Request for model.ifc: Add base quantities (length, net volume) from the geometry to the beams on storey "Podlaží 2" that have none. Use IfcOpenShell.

First a look at what the model holds.

```python
import ifcopenshell
import ifcopenshell.util.element
import ifcopenshell.util.unit

model = ifcopenshell.open("model.ifc")
print(model.schema)
for unit_type in ("LENGTHUNIT", "AREAUNIT", "VOLUMEUNIT"):
    print(unit_type, ifcopenshell.util.unit.calculate_unit_scale(model, unit_type))
storey = next(s for s in model.by_type("IfcBuildingStorey") if s.Name == "Podlaží 2")
beams = [e for e in ifcopenshell.util.element.get_decomposition(storey) if e.is_a("IfcBeam")]
for e in sorted(beams, key=lambda e: e.id()):
    print(e.id(), e.is_a(), e.Name, list(ifcopenshell.util.element.get_psets(e, qtos_only=True)), sep=" | ")
```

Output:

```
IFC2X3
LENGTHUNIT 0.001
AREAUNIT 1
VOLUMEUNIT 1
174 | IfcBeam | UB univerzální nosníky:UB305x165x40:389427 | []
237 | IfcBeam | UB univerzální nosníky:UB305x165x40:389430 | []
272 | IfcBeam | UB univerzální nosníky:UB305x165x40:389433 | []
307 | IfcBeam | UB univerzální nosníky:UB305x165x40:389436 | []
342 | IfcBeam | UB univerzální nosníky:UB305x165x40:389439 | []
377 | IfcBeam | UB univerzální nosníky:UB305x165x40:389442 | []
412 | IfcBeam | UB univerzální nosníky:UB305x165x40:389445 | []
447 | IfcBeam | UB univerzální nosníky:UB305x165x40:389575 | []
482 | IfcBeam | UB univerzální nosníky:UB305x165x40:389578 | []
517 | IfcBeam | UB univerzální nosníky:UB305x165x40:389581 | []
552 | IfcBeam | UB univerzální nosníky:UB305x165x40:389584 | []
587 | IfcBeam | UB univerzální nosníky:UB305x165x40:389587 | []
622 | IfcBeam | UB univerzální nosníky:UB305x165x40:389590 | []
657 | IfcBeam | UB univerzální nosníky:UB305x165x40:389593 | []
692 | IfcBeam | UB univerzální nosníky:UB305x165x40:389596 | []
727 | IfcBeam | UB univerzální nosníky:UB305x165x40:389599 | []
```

```python
import ifcopenshell
import ifcopenshell.api.pset
import ifcopenshell.geom
import ifcopenshell.util.element
import ifcopenshell.util.shape
import ifcopenshell.util.unit

model = ifcopenshell.open("model.ifc")
unit_scale = ifcopenshell.util.unit.calculate_unit_scale(model)
volume_scale = ifcopenshell.util.unit.calculate_unit_scale(model, "VOLUMEUNIT")
settings = ifcopenshell.geom.settings()

storey = next(s for s in model.by_type("IfcBuildingStorey") if s.Name == "Podlaží 2")
beams = [e for e in ifcopenshell.util.element.get_decomposition(storey) if e.is_a("IfcBeam")]

for e in sorted(beams, key=lambda e: e.id()):
    if ifcopenshell.util.element.get_psets(e, qtos_only=True, should_inherit=False):
        continue
    # Geometry comes back in metres, in the element's own axes.
    shape = ifcopenshell.geom.create_shape(settings, e)
    values = {
        "Length": ifcopenshell.util.shape.get_max_xyz(shape.geometry) / unit_scale,
        "NetVolume": ifcopenshell.util.shape.get_volume(shape.geometry) / volume_scale,
    }
    qto = ifcopenshell.api.pset.add_qto(model, product=e, name="BaseQuantities")
    ifcopenshell.api.pset.edit_qto(model, qto=qto, properties=values)
    print(e.id(), {k: round(v, 3) for k, v in values.items()})

model.write("model_v2.ifc")
```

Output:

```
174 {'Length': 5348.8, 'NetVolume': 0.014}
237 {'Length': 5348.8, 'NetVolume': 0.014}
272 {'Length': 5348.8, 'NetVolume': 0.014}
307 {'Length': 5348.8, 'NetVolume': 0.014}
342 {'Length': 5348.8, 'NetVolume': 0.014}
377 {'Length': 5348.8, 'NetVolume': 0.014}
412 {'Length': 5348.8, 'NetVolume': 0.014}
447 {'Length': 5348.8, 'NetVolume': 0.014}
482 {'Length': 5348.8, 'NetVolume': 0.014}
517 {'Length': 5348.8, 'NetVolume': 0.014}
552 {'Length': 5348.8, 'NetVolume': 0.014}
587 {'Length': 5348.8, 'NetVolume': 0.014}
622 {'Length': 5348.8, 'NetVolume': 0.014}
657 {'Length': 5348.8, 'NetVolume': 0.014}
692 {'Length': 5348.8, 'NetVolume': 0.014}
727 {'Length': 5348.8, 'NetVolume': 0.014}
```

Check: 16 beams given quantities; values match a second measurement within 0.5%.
